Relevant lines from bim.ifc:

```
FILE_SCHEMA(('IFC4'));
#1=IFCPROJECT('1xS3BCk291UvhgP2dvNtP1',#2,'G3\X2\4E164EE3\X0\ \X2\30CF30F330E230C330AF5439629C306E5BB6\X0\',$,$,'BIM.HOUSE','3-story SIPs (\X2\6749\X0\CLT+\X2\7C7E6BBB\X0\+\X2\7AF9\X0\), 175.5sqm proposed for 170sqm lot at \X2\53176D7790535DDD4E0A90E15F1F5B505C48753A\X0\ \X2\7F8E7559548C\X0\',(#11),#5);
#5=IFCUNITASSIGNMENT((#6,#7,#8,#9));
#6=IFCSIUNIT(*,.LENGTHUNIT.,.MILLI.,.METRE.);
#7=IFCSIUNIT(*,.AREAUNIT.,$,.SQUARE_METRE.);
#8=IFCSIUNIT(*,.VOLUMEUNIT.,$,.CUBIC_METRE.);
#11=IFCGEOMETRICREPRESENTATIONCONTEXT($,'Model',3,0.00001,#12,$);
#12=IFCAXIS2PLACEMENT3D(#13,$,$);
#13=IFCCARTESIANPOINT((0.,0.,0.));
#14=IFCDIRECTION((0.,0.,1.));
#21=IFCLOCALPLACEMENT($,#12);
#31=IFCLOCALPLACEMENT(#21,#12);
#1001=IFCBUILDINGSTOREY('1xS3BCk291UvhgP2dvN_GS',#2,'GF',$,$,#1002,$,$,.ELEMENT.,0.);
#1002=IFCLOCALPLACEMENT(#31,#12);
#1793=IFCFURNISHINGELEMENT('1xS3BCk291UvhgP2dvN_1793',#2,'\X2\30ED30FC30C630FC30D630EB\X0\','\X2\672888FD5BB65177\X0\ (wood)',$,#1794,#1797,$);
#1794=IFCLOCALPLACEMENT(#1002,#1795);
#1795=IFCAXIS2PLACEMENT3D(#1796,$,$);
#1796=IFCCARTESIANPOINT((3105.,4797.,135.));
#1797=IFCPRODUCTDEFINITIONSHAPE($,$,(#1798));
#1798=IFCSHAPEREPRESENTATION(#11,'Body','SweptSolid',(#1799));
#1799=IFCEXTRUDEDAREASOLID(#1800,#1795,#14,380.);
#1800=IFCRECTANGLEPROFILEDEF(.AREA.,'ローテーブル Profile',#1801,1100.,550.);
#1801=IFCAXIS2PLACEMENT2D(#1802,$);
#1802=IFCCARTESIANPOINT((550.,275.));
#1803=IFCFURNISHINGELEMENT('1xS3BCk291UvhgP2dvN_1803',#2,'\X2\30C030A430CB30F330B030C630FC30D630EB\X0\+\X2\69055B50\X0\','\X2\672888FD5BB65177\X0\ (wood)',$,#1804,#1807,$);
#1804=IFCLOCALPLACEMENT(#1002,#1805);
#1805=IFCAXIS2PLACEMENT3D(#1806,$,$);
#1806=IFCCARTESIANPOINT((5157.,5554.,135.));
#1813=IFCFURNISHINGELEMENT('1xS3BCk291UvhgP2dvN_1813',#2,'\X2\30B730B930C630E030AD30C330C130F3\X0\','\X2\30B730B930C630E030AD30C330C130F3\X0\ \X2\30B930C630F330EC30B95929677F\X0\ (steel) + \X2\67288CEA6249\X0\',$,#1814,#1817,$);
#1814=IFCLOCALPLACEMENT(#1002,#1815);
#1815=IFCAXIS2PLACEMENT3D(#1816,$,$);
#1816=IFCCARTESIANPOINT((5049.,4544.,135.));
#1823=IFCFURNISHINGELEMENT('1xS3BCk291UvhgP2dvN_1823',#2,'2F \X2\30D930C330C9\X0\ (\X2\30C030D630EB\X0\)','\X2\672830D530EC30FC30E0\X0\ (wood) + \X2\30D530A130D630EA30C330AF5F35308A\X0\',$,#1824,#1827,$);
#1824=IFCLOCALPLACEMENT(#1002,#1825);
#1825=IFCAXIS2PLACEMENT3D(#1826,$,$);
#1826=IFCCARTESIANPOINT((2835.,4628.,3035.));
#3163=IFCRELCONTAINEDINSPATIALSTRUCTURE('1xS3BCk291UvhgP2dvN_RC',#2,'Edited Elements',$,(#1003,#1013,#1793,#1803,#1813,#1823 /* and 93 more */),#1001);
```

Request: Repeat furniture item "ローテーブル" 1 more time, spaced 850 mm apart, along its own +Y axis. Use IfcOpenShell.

```python
import ifcopenshell
import ifcopenshell.api.geometry
import ifcopenshell.api.root
import ifcopenshell.util.element
import ifcopenshell.util.placement
import ifcopenshell.util.unit

model = ifcopenshell.open("bim.ifc")
unit_scale = ifcopenshell.util.unit.calculate_unit_scale(model)


def reuse_history(source, copy):
    """copy_class also copies each property set's owner history, people and application; keep the originals."""
    for rel in copy.IsDefinedBy:
        if rel.is_a("IfcRelDefinesByProperties") and (history := rel.RelatingPropertyDefinition.OwnerHistory):
            rel.RelatingPropertyDefinition.OwnerHistory = source.OwnerHistory
            ifcopenshell.util.element.remove_deep2(model, history)


source = model.by_guid("1xS3BCk291UvhgP2dvN_1793")
base = ifcopenshell.util.placement.get_local_placement(source.ObjectPlacement)
step = base[:3, 1] * 0.85 / unit_scale

for i in range(1, 2):
    copy = ifcopenshell.api.root.copy_class(model, product=source)
    copy.Representation = ifcopenshell.util.element.copy_deep(
        model, source.Representation, exclude=["IfcGeometricRepresentationContext", "IfcRepresentationMap"]
    )
    reuse_history(source, copy)
    matrix = base.copy()
    matrix[:3, 3] += i * step
    print("added at", matrix[:3, 3].round(3) + 0.0)
    ifcopenshell.api.geometry.edit_object_placement(model, product=copy, matrix=matrix, is_si=False)

model.write("bim-out.ifc")
```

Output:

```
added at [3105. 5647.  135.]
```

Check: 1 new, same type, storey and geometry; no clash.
